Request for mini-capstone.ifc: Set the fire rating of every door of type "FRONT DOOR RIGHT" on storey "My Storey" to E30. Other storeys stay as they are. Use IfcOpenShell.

First a look at what the model holds.

```python
import ifcopenshell
import ifcopenshell.util.element

model = ifcopenshell.open("mini-capstone.ifc")
print(model.schema)
storey = next(s for s in model.by_type("IfcBuildingStorey") if s.Name == "My Storey")
doors = [e for e in ifcopenshell.util.element.get_decomposition(storey) if e.is_a("IfcDoor")]
seen = {}
for e in doors:
    element_type = ifcopenshell.util.element.get_type(e)
    key = (element_type.Name if element_type != e and element_type else None, ifcopenshell.util.element.get_pset(e, "Pset_DoorCommon", "FireRating"))
    seen[key] = seen.get(key, 0) + 1
for (name, value), count in sorted(seen.items(), key=str):
    print(count, "x", name, "|", value)
```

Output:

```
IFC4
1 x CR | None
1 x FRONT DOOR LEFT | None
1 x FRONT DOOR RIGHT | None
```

```python
import ifcopenshell
import ifcopenshell.api.pset
import ifcopenshell.util.element

model = ifcopenshell.open("mini-capstone.ifc")

storey = next(s for s in model.by_type("IfcBuildingStorey") if s.Name == "My Storey")
doors = [e for e in ifcopenshell.util.element.get_decomposition(storey) if e.is_a("IfcDoor")]

count = 0
for e in doors:
    element_type = ifcopenshell.util.element.get_type(e)
    if element_type in (None, e) or element_type.Name != "FRONT DOOR RIGHT":
        continue
    # add_pset returns the element's existing set when there is one.
    pset = ifcopenshell.api.pset.add_pset(model, product=e, name="Pset_DoorCommon")
    ifcopenshell.api.pset.edit_pset(model, pset=pset, properties={"FireRating": "E30"})
    count += 1

print(count, "doors updated")

model.write("mini-capstone_edited.ifc")
```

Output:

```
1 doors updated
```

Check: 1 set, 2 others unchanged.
